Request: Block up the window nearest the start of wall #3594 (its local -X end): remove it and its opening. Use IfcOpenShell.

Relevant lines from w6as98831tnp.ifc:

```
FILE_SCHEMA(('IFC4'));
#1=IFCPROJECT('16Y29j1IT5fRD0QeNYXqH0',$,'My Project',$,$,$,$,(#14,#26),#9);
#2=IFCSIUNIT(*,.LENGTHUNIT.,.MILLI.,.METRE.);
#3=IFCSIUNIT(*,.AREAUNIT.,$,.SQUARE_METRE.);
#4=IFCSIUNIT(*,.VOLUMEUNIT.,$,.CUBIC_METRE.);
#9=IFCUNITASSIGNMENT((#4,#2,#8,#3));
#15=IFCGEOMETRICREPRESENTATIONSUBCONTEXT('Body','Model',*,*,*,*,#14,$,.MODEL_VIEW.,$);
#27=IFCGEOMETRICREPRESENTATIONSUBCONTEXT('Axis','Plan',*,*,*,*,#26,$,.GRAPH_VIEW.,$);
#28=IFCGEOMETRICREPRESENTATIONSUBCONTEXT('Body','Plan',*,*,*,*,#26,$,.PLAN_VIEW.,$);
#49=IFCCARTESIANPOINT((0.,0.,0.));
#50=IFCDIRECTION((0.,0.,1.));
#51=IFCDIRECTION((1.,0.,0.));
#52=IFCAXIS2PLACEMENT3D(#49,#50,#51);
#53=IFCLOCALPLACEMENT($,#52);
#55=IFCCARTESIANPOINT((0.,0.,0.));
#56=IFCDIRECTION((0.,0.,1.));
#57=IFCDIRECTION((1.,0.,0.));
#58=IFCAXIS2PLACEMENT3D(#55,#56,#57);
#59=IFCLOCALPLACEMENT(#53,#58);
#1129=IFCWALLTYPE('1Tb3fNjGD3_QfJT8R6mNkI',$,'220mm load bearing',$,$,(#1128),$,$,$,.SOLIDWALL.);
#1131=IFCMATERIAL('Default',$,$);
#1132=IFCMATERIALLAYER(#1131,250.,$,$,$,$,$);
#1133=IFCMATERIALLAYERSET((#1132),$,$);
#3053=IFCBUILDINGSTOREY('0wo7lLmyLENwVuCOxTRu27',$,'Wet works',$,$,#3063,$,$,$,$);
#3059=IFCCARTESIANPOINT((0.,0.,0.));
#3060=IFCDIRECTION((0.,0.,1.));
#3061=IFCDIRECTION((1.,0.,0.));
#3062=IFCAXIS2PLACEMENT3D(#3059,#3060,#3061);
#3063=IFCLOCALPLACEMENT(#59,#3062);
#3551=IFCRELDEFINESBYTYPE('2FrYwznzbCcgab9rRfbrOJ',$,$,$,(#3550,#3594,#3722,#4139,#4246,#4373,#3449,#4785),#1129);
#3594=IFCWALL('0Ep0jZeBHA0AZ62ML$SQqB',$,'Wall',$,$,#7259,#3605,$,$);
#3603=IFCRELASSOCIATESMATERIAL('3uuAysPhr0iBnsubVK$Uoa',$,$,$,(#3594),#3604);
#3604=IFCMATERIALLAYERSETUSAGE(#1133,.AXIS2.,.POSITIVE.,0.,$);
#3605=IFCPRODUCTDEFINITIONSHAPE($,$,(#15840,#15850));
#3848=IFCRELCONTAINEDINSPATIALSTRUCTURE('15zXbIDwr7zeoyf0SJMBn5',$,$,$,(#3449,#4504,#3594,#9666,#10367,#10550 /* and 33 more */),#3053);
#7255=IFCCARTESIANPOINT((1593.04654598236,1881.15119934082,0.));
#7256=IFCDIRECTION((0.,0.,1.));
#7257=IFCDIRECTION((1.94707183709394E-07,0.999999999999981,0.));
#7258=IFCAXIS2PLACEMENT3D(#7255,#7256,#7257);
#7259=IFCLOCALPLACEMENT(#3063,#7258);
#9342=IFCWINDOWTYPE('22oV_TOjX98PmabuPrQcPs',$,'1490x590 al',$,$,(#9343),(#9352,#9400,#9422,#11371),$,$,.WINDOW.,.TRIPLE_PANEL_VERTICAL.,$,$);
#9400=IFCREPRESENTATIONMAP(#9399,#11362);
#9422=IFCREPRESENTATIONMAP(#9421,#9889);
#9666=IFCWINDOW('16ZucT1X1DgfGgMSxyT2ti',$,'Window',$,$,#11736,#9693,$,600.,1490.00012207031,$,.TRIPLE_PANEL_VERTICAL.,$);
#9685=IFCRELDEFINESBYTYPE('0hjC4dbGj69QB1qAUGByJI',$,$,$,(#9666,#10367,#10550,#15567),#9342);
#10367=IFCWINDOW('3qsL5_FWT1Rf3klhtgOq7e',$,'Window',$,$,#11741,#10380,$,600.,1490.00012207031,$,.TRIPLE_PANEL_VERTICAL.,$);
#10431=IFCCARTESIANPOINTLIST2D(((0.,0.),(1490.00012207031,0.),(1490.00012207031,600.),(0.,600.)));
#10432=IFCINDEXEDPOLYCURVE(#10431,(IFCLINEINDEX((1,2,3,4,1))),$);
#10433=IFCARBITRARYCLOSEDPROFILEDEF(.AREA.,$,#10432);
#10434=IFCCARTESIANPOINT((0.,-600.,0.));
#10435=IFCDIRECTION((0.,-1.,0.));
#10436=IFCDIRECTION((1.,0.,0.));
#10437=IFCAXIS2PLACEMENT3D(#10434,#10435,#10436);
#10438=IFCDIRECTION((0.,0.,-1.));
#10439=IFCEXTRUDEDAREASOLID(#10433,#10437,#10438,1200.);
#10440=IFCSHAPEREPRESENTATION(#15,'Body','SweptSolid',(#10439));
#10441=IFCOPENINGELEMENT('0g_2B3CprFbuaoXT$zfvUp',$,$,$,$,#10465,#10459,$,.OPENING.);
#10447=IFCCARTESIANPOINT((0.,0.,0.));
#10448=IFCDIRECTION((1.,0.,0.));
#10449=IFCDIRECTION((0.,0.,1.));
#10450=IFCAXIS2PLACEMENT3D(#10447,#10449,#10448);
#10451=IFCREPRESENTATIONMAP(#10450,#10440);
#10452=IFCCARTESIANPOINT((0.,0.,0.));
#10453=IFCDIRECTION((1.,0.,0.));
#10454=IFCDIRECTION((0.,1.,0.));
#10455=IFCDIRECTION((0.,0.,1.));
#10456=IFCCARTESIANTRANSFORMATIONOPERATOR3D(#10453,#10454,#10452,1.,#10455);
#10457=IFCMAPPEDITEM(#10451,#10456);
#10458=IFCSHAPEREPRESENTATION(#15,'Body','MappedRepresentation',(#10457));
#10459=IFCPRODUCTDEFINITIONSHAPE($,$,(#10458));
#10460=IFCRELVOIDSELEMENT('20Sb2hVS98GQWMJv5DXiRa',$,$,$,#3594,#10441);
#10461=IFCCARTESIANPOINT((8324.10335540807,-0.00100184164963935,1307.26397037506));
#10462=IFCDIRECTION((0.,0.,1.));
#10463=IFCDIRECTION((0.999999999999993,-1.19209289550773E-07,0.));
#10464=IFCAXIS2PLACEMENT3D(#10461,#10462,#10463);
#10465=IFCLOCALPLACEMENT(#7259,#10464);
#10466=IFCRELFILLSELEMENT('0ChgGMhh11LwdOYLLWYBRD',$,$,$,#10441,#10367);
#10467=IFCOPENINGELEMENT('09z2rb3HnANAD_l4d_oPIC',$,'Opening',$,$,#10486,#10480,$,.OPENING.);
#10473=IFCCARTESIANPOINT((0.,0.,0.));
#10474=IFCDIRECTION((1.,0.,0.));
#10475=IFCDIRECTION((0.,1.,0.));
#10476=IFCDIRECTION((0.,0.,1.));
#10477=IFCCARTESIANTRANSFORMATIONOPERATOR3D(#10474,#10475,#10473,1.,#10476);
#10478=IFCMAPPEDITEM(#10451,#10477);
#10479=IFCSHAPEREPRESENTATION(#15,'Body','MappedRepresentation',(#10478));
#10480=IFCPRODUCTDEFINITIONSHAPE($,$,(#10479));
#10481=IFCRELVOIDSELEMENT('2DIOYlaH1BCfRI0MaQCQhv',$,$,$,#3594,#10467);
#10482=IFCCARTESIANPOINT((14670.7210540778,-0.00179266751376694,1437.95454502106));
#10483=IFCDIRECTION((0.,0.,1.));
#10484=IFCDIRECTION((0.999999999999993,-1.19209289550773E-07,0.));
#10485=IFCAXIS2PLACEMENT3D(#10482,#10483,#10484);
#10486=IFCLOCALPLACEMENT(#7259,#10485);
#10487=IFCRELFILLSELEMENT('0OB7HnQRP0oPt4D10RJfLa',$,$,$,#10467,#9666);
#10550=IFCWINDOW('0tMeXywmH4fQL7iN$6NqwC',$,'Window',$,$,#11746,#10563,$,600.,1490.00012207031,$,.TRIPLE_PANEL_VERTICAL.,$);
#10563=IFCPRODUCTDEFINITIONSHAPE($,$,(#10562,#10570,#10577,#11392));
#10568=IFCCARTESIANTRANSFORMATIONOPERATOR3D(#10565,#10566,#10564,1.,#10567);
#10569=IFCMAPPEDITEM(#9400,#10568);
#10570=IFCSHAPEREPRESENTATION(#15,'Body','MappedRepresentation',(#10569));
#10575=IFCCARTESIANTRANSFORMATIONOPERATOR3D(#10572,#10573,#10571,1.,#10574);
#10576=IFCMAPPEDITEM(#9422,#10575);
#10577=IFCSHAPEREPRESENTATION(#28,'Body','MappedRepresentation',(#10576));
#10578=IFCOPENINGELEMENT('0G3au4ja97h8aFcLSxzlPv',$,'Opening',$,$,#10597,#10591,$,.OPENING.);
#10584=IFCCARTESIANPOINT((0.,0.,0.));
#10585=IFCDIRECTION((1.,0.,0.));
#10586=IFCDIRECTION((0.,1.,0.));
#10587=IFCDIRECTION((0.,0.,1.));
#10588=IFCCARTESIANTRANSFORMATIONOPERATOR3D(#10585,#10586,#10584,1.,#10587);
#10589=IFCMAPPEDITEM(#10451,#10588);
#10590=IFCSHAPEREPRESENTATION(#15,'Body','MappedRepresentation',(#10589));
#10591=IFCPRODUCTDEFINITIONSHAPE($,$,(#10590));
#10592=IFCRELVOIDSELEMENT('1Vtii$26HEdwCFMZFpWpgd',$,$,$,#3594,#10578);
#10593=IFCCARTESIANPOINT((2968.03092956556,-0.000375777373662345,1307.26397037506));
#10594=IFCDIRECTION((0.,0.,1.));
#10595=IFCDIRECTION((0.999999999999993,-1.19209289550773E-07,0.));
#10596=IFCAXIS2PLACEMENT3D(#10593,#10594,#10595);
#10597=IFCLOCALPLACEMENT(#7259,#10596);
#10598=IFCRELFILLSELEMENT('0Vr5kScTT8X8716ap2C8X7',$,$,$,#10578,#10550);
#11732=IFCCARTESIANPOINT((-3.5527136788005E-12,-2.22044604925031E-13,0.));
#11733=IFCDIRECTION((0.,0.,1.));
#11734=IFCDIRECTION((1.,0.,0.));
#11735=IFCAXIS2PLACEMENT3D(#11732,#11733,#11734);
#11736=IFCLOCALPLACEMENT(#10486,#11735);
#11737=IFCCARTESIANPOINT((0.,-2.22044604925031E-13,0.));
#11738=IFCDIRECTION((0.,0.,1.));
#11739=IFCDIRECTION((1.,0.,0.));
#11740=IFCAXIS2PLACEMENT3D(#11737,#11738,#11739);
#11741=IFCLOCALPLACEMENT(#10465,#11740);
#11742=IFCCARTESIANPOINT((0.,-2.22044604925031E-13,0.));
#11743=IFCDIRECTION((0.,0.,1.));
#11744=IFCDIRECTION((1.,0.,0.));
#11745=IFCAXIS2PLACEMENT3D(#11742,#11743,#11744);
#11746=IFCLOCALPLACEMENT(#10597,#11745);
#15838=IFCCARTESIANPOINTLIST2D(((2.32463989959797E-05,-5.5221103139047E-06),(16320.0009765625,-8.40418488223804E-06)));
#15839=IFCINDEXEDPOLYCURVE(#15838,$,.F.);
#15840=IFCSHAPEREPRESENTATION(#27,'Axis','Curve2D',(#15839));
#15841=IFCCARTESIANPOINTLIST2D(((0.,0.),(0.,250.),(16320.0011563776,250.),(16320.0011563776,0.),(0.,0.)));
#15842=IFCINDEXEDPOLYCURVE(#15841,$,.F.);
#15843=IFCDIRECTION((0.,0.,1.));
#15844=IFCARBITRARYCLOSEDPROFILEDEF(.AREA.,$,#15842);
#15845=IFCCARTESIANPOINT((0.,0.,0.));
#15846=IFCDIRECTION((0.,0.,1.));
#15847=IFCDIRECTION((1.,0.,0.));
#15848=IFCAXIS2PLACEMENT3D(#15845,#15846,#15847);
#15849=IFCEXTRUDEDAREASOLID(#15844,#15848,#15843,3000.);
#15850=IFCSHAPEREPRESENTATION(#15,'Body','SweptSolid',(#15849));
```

```python
import ifcopenshell
import ifcopenshell.api.feature
import ifcopenshell.api.root
import ifcopenshell.geom
import ifcopenshell.util.shape

model = ifcopenshell.open("w6as98831tnp.ifc")
settings = ifcopenshell.geom.settings()


def volume(element):
    """Net volume in cubic metres, openings subtracted."""
    shape = ifcopenshell.geom.create_shape(settings, element)
    return ifcopenshell.util.shape.get_volume(shape.geometry)


window = model.by_guid("0tMeXywmH4fQL7iN$6NqwC")
opening = window.FillsVoids[0].RelatingOpeningElement
wall = opening.VoidsElements[0].RelatingBuildingElement
before = volume(wall)

ifcopenshell.api.root.remove_product(model, product=window)
ifcopenshell.api.feature.remove_feature(model, feature=opening)

after = volume(wall)

print(f"wall volume {before:.3f} -> {after:.3f} m3")

model.write("w6as98831tnp-out.ifc")
```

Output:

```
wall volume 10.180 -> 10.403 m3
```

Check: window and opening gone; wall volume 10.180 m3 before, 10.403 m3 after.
